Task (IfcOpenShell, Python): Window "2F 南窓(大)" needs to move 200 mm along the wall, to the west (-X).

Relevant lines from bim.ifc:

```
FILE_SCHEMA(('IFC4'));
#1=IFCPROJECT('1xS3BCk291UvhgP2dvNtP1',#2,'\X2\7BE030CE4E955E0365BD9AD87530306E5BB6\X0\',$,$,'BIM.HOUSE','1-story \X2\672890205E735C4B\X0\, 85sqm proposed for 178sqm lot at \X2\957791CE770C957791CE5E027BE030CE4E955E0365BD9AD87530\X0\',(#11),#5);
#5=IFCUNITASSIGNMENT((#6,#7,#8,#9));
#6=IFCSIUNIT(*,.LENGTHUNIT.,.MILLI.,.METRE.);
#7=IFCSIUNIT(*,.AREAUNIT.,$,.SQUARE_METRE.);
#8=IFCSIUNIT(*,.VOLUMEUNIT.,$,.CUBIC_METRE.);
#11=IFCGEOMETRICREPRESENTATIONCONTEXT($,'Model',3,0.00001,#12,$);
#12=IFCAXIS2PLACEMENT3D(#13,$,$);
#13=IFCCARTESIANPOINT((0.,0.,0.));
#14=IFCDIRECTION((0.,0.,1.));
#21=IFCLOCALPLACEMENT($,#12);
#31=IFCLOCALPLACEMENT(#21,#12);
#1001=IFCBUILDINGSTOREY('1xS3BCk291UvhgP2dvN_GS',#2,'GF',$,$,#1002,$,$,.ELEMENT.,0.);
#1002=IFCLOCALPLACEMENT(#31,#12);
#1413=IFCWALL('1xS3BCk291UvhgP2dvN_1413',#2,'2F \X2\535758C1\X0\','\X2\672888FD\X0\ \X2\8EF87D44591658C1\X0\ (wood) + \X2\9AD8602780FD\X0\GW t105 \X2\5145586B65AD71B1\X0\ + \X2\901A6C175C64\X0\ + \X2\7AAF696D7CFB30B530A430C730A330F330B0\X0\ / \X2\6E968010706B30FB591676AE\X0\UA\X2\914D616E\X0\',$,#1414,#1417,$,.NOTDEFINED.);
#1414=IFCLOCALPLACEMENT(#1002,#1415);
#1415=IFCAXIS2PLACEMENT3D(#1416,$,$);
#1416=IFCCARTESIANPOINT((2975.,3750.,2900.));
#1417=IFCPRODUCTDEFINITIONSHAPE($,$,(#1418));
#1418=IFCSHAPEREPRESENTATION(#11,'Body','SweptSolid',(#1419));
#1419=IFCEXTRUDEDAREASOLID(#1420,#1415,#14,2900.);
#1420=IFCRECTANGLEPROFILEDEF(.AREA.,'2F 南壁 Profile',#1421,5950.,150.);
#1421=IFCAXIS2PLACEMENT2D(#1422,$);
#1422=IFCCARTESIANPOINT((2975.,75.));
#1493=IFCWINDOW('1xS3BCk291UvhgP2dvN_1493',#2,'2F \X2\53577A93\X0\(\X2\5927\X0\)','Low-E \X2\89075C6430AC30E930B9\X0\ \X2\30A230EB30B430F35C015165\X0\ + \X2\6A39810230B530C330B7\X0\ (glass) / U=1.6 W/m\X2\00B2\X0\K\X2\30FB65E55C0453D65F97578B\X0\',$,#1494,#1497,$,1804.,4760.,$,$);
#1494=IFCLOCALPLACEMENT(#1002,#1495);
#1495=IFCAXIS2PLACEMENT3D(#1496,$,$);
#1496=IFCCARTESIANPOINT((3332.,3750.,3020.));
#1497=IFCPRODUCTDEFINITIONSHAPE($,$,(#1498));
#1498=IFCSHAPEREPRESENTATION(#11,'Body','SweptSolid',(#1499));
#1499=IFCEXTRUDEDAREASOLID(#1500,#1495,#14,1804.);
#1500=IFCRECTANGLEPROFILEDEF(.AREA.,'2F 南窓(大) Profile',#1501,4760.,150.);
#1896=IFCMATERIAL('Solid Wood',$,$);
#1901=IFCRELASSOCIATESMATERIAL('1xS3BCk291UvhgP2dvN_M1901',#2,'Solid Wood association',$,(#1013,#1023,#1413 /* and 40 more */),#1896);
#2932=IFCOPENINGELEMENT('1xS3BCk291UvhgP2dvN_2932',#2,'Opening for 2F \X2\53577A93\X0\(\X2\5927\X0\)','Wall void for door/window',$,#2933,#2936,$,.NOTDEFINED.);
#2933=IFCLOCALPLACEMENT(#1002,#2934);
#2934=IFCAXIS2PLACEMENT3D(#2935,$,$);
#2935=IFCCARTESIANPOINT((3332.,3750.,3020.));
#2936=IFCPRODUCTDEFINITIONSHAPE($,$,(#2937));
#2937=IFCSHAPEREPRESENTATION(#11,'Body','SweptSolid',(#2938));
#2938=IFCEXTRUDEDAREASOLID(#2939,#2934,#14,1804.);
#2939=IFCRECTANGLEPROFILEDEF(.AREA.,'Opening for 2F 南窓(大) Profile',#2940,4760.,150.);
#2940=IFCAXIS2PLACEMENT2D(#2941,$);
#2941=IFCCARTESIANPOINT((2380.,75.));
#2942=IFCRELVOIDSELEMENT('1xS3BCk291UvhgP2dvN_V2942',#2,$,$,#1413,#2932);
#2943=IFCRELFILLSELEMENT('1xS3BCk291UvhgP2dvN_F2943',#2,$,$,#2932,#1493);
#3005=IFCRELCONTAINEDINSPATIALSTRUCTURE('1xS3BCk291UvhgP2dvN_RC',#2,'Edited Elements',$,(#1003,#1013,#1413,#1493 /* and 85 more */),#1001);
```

```python
import ifcopenshell
import ifcopenshell.api.geometry
import ifcopenshell.util.placement
import ifcopenshell.util.unit

model = ifcopenshell.open("bim.ifc")
unit_scale = ifcopenshell.util.unit.calculate_unit_scale(model)

window = model.by_guid("1xS3BCk291UvhgP2dvN_1493")
opening = window.FillsVoids[0].RelatingOpeningElement
wall = opening.VoidsElements[0].RelatingBuildingElement

wall_matrix = ifcopenshell.util.placement.get_local_placement(wall.ObjectPlacement)
shift = wall_matrix[:3, 0] * -0.2 / unit_scale
before = ifcopenshell.util.placement.get_local_placement(window.ObjectPlacement)[:3, 3].copy()

# The window is not placed relative to its opening, so move both.
for product in (opening, window):
    matrix = ifcopenshell.util.placement.get_local_placement(product.ObjectPlacement)
    matrix[:3, 3] += shift
    ifcopenshell.api.geometry.edit_object_placement(model, product=product, matrix=matrix, is_si=False)

after = ifcopenshell.util.placement.get_local_placement(window.ObjectPlacement)[:3, 3]
print("window moved by", (after - before).round(3) + 0.0)

model.write("bim_rev.ifc")
```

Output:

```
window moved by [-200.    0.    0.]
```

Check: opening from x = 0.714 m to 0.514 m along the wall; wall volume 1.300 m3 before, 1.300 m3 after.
